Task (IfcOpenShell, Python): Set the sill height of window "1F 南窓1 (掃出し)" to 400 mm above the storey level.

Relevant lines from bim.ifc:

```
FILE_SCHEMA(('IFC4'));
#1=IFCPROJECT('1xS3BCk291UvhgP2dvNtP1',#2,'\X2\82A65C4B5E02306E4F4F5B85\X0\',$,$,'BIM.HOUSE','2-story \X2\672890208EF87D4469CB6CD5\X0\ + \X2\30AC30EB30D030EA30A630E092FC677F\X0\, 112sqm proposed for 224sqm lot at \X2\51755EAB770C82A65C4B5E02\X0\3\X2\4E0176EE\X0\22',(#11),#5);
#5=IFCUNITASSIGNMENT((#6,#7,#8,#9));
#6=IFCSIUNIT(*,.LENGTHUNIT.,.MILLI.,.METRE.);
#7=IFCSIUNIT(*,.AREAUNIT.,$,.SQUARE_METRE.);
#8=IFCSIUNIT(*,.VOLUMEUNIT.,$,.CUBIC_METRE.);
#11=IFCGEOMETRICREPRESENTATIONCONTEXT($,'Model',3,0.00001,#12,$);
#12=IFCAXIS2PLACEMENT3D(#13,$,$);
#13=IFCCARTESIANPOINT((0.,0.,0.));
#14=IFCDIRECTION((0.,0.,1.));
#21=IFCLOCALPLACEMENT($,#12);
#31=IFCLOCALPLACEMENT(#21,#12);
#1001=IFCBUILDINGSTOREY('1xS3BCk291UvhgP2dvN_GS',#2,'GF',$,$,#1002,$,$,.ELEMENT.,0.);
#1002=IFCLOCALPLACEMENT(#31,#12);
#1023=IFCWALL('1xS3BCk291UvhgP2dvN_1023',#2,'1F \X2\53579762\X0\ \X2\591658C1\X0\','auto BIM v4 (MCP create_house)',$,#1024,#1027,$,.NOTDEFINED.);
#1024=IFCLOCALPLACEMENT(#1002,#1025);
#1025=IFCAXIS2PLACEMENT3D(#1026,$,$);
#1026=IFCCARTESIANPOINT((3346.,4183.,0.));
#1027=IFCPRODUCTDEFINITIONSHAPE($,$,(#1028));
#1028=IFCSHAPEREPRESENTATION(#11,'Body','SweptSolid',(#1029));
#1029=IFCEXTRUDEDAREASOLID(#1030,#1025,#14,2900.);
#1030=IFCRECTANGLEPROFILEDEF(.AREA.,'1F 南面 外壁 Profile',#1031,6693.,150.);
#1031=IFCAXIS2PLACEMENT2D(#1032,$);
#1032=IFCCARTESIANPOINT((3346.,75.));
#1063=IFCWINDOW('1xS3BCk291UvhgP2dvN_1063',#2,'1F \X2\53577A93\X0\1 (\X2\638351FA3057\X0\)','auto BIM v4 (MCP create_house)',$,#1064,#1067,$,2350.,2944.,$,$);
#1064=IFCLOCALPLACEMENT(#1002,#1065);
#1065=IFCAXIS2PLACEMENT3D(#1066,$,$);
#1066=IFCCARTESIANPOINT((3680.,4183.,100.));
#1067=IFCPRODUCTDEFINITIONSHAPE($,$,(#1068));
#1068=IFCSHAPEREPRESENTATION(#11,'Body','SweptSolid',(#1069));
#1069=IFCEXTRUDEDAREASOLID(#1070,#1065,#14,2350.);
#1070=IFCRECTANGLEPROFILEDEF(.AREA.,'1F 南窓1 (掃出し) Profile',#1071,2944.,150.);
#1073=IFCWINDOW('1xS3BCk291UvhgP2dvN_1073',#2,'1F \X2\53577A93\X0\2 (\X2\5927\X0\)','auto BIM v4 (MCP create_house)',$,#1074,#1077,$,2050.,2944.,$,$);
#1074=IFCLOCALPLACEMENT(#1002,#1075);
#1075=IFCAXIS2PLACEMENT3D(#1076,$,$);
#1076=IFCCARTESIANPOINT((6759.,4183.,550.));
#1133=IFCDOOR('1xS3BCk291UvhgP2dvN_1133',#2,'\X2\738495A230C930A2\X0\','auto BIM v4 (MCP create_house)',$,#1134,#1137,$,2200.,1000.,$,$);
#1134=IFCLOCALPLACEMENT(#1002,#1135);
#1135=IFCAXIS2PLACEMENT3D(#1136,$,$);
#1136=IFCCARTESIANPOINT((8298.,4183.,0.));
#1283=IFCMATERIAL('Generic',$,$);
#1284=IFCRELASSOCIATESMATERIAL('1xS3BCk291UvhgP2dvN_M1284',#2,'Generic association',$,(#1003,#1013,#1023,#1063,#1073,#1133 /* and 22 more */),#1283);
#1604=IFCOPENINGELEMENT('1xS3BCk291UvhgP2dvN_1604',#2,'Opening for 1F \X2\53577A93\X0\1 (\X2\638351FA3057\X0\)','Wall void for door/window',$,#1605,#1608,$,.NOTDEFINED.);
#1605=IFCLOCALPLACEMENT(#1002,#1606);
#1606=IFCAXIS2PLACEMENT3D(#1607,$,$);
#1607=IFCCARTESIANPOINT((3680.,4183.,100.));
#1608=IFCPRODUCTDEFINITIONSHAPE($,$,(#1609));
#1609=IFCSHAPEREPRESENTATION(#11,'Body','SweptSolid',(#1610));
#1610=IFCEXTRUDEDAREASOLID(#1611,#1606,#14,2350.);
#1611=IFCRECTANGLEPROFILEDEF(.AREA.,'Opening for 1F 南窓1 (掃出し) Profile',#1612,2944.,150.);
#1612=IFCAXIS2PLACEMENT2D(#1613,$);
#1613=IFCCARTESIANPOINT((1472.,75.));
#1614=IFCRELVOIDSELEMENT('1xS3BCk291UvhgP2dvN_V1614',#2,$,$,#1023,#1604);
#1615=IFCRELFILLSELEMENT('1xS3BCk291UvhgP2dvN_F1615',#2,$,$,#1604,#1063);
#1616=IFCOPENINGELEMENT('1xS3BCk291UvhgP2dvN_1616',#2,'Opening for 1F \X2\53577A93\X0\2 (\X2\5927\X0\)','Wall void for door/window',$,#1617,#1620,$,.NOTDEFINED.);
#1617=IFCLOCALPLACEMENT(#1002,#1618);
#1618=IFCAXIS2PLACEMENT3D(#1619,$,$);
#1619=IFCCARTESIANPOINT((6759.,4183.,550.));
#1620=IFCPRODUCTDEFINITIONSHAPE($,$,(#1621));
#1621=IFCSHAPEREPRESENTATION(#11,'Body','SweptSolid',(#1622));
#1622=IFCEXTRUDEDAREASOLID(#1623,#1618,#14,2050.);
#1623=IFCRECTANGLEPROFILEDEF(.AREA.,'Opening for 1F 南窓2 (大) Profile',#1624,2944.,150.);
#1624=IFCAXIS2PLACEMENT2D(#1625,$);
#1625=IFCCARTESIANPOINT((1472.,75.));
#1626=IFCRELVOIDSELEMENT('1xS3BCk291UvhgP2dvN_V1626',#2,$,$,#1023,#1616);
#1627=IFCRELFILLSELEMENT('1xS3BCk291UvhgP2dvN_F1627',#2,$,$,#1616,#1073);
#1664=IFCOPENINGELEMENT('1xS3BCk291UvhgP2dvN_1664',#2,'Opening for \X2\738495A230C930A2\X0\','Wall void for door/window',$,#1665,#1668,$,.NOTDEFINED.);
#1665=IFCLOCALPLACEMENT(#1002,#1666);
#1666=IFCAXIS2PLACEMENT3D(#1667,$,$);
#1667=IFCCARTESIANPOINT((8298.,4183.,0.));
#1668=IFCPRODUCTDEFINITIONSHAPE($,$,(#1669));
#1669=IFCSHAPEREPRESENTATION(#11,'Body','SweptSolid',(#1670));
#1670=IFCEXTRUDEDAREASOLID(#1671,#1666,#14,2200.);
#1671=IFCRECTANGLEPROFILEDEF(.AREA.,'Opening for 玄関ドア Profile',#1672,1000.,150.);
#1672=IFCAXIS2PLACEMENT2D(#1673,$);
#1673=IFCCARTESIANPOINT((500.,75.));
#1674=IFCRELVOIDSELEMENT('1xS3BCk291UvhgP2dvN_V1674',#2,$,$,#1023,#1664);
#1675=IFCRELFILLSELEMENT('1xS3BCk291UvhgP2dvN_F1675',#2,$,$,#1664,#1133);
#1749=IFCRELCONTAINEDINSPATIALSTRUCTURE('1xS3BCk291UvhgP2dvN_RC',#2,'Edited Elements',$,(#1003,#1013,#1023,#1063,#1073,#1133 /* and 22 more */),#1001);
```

```python
import numpy as np
import ifcopenshell
import ifcopenshell.api.geometry
import ifcopenshell.geom
import ifcopenshell.util.element
import ifcopenshell.util.placement
import ifcopenshell.util.shape
import ifcopenshell.util.unit

model = ifcopenshell.open("bim.ifc")
unit_scale = ifcopenshell.util.unit.calculate_unit_scale(model)

window = model.by_guid("1xS3BCk291UvhgP2dvN_1063")
opening = window.FillsVoids[0].RelatingOpeningElement
storey = ifcopenshell.util.element.get_container(window, ifc_class="IfcBuildingStorey")
level = ifcopenshell.util.placement.get_local_placement(storey.ObjectPlacement)[2, 3]

# The opening's origin need not be at the sill, so measure its lowest point.
shape = ifcopenshell.geom.create_shape(ifcopenshell.geom.settings(), opening)
bottom = ifcopenshell.util.shape.get_shape_bottom_elevation(shape, shape.geometry) / unit_scale
dz = level + 0.4 / unit_scale - bottom

shift = np.array([0.0, 0.0, dz])
# The window is not placed relative to its opening, so move both.
for product in (opening, window):
    matrix = ifcopenshell.util.placement.get_local_placement(product.ObjectPlacement)
    matrix[:3, 3] += shift
    ifcopenshell.api.geometry.edit_object_placement(model, product=product, matrix=matrix, is_si=False)

print(f"moved by {dz * unit_scale:+.3f} m")

model.write("bim_rev.ifc")
```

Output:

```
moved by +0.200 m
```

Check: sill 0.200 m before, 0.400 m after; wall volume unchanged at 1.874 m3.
